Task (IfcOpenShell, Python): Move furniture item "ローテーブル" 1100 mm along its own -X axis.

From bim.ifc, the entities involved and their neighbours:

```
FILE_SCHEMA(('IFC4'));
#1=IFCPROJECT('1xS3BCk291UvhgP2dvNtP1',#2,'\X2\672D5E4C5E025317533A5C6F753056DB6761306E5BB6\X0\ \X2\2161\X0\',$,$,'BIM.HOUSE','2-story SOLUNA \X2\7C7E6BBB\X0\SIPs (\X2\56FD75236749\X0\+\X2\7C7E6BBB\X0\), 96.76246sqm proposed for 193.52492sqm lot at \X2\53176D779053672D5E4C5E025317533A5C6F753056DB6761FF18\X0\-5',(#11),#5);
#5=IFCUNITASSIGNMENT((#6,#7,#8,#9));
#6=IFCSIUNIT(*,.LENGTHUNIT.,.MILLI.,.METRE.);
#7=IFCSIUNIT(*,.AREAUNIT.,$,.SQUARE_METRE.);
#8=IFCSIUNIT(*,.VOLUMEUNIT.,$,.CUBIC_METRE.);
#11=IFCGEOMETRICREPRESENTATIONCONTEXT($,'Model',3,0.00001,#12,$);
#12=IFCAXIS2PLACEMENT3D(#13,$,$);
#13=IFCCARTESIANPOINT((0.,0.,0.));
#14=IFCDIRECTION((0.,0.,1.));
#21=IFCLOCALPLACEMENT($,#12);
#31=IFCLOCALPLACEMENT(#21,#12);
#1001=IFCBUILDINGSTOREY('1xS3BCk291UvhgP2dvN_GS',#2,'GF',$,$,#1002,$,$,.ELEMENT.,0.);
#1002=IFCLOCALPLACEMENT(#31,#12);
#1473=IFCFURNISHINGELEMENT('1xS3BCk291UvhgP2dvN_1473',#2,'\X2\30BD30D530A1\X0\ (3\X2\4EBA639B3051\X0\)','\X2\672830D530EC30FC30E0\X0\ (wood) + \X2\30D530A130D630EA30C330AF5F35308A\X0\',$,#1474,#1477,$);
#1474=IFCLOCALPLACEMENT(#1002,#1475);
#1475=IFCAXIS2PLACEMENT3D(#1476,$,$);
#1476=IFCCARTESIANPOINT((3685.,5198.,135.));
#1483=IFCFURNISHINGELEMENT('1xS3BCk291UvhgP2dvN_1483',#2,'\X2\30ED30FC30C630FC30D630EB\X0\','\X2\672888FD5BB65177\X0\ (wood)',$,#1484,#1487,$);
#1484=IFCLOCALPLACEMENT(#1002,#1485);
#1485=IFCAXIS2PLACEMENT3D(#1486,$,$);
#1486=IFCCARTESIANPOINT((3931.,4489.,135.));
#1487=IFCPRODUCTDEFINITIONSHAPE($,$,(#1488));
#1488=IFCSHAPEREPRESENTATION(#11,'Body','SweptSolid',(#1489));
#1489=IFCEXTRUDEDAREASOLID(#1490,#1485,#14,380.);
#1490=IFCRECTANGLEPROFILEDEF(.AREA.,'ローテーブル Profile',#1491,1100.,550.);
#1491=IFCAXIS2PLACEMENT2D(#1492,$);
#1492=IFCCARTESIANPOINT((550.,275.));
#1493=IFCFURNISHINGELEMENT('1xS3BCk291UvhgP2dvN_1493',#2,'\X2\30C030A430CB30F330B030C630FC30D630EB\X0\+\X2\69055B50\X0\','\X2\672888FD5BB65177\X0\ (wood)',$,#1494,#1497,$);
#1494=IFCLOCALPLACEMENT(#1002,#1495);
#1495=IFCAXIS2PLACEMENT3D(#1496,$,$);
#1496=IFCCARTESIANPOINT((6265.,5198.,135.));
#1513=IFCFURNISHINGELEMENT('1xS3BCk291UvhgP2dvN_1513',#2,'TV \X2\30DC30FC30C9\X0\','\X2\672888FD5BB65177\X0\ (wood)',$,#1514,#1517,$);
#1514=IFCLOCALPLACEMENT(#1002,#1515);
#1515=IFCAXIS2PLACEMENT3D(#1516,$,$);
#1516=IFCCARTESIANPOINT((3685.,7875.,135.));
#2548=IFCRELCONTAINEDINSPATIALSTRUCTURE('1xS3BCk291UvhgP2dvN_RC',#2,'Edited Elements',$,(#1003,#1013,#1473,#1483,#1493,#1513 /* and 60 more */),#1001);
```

```python
import ifcopenshell
import ifcopenshell.api.geometry
import ifcopenshell.util.placement
import ifcopenshell.util.unit

model = ifcopenshell.open("bim.ifc")
unit_scale = ifcopenshell.util.unit.calculate_unit_scale(model)

item = model.by_guid("1xS3BCk291UvhgP2dvN_1483")
matrix = ifcopenshell.util.placement.get_local_placement(item.ObjectPlacement)
matrix[:3, 3] -= matrix[:3, 0] * 1.1 / unit_scale
ifcopenshell.api.geometry.edit_object_placement(model, product=item, matrix=matrix, is_si=False)

print(ifcopenshell.util.placement.get_local_placement(item.ObjectPlacement).round(3) + 0.0)

model.write("bim_v2.ifc")
```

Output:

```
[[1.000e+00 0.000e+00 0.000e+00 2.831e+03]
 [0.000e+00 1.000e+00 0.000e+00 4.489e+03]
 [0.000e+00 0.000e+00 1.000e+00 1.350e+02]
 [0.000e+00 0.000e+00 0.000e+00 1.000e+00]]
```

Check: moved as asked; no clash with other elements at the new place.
